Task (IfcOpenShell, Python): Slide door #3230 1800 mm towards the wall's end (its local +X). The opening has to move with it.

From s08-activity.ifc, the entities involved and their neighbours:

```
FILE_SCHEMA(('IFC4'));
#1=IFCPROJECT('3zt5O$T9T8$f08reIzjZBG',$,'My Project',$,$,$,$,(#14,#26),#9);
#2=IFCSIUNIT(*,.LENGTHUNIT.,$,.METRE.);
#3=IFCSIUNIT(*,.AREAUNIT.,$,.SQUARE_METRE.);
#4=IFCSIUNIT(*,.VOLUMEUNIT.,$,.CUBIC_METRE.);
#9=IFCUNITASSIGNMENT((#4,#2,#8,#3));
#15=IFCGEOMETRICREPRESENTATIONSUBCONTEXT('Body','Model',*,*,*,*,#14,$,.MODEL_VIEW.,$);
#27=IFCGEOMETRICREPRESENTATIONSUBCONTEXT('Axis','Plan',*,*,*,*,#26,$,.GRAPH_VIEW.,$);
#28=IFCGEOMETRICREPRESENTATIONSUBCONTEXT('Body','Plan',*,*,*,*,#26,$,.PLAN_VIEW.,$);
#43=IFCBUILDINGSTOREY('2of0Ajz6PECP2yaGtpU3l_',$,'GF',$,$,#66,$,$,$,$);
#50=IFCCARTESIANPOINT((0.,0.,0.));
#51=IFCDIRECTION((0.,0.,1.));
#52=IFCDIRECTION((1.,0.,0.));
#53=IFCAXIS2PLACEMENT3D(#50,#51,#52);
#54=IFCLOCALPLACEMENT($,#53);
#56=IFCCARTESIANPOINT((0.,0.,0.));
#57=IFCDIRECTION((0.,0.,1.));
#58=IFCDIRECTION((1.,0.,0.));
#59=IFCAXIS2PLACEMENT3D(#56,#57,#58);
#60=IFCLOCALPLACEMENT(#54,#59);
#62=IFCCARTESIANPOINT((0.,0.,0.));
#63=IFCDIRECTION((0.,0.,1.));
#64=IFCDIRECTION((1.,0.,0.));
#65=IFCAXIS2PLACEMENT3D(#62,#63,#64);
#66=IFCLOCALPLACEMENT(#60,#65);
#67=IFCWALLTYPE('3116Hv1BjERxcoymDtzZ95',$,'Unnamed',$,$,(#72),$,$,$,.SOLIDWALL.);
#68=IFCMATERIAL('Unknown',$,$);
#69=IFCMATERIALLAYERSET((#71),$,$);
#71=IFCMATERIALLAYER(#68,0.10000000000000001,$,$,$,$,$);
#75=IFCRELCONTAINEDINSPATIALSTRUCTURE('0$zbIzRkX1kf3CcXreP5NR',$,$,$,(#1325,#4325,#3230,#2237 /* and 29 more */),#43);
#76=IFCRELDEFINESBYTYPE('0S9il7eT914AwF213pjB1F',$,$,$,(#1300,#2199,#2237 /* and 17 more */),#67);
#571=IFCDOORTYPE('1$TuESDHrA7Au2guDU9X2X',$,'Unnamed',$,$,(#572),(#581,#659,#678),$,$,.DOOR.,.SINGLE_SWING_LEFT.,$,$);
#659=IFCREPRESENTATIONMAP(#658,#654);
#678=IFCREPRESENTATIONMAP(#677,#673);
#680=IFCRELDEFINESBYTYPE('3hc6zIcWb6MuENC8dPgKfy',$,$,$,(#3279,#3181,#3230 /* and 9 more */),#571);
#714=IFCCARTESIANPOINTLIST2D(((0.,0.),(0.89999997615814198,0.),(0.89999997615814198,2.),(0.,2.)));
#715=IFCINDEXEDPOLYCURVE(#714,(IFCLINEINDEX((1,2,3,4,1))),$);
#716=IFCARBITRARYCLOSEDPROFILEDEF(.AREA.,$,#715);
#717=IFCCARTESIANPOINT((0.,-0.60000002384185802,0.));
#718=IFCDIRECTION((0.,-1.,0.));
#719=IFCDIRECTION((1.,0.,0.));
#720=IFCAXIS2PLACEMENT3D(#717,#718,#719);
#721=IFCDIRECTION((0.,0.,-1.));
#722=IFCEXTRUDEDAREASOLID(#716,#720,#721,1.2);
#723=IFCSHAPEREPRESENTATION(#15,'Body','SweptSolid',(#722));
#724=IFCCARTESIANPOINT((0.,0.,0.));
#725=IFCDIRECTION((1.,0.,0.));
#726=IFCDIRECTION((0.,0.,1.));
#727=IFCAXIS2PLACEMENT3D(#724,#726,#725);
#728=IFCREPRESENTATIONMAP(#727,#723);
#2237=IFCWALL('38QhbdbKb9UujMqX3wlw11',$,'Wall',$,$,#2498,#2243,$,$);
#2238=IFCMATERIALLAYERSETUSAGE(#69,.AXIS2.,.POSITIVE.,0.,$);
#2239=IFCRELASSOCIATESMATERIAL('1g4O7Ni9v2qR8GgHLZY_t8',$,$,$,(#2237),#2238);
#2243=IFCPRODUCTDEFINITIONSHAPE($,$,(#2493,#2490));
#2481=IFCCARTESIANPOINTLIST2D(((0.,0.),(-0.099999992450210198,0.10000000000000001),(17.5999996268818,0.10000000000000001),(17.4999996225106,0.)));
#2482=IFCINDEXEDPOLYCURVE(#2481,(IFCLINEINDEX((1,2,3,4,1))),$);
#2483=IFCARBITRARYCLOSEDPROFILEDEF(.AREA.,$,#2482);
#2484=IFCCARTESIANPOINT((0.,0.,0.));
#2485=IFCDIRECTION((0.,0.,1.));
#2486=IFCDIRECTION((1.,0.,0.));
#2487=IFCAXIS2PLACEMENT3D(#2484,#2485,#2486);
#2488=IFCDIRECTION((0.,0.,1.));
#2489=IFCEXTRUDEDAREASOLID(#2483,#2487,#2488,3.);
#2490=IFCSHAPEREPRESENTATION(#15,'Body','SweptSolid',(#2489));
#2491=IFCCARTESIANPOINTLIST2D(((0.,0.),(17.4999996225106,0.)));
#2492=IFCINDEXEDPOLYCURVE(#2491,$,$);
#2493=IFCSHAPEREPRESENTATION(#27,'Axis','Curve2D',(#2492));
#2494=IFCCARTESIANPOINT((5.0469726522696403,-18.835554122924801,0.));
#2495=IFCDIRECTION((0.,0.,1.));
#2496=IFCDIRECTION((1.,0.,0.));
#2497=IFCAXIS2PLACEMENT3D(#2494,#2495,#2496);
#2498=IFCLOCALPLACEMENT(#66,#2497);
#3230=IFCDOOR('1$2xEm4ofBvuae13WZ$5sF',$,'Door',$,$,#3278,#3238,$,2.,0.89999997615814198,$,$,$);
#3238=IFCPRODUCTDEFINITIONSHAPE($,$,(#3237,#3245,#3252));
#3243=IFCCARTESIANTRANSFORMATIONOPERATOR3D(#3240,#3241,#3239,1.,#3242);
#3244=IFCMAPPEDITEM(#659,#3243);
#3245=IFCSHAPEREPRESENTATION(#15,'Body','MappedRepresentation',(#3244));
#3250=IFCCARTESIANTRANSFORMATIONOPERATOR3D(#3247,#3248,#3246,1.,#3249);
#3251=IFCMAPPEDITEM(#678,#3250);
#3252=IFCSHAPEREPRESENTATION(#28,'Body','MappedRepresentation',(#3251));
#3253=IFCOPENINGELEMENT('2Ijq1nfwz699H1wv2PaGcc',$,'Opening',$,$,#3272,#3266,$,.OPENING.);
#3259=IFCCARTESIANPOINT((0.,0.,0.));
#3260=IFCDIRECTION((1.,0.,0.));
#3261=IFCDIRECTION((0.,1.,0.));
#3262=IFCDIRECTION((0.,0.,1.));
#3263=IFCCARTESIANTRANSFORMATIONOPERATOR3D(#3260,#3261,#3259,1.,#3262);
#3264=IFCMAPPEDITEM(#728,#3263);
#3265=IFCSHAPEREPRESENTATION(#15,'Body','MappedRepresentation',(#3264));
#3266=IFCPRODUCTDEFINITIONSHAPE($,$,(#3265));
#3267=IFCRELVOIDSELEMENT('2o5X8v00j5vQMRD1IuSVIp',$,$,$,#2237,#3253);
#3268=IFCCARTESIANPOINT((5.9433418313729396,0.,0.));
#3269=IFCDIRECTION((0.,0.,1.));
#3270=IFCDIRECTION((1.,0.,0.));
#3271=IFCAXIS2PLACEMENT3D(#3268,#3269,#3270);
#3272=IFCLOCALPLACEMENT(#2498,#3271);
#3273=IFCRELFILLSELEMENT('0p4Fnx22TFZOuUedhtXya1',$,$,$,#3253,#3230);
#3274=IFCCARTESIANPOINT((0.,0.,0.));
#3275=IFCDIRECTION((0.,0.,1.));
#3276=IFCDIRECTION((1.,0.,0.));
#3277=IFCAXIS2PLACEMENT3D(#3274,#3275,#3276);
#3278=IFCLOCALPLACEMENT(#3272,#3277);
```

```python
import ifcopenshell
import ifcopenshell.api.geometry
import ifcopenshell.util.placement

model = ifcopenshell.open("s08-activity.ifc")

door = model.by_guid("1$2xEm4ofBvuae13WZ$5sF")
opening = door.FillsVoids[0].RelatingOpeningElement
wall = opening.VoidsElements[0].RelatingBuildingElement

wall_matrix = ifcopenshell.util.placement.get_local_placement(wall.ObjectPlacement)
shift = wall_matrix[:3, 0] * 1.8
before = ifcopenshell.util.placement.get_local_placement(door.ObjectPlacement)[:3, 3].copy()

# The door is placed relative to its opening, so it follows when the opening moves.
matrix = ifcopenshell.util.placement.get_local_placement(opening.ObjectPlacement)
matrix[:3, 3] += shift
ifcopenshell.api.geometry.edit_object_placement(
    model, product=opening, matrix=matrix, is_si=False, should_transform_children=True
)

after = ifcopenshell.util.placement.get_local_placement(door.ObjectPlacement)[:3, 3]
print("door moved by", (after - before).round(3) + 0.0)

model.write("s08-activity_rev.ifc")
```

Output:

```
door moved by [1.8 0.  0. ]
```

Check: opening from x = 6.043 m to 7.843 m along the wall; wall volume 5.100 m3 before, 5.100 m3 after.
